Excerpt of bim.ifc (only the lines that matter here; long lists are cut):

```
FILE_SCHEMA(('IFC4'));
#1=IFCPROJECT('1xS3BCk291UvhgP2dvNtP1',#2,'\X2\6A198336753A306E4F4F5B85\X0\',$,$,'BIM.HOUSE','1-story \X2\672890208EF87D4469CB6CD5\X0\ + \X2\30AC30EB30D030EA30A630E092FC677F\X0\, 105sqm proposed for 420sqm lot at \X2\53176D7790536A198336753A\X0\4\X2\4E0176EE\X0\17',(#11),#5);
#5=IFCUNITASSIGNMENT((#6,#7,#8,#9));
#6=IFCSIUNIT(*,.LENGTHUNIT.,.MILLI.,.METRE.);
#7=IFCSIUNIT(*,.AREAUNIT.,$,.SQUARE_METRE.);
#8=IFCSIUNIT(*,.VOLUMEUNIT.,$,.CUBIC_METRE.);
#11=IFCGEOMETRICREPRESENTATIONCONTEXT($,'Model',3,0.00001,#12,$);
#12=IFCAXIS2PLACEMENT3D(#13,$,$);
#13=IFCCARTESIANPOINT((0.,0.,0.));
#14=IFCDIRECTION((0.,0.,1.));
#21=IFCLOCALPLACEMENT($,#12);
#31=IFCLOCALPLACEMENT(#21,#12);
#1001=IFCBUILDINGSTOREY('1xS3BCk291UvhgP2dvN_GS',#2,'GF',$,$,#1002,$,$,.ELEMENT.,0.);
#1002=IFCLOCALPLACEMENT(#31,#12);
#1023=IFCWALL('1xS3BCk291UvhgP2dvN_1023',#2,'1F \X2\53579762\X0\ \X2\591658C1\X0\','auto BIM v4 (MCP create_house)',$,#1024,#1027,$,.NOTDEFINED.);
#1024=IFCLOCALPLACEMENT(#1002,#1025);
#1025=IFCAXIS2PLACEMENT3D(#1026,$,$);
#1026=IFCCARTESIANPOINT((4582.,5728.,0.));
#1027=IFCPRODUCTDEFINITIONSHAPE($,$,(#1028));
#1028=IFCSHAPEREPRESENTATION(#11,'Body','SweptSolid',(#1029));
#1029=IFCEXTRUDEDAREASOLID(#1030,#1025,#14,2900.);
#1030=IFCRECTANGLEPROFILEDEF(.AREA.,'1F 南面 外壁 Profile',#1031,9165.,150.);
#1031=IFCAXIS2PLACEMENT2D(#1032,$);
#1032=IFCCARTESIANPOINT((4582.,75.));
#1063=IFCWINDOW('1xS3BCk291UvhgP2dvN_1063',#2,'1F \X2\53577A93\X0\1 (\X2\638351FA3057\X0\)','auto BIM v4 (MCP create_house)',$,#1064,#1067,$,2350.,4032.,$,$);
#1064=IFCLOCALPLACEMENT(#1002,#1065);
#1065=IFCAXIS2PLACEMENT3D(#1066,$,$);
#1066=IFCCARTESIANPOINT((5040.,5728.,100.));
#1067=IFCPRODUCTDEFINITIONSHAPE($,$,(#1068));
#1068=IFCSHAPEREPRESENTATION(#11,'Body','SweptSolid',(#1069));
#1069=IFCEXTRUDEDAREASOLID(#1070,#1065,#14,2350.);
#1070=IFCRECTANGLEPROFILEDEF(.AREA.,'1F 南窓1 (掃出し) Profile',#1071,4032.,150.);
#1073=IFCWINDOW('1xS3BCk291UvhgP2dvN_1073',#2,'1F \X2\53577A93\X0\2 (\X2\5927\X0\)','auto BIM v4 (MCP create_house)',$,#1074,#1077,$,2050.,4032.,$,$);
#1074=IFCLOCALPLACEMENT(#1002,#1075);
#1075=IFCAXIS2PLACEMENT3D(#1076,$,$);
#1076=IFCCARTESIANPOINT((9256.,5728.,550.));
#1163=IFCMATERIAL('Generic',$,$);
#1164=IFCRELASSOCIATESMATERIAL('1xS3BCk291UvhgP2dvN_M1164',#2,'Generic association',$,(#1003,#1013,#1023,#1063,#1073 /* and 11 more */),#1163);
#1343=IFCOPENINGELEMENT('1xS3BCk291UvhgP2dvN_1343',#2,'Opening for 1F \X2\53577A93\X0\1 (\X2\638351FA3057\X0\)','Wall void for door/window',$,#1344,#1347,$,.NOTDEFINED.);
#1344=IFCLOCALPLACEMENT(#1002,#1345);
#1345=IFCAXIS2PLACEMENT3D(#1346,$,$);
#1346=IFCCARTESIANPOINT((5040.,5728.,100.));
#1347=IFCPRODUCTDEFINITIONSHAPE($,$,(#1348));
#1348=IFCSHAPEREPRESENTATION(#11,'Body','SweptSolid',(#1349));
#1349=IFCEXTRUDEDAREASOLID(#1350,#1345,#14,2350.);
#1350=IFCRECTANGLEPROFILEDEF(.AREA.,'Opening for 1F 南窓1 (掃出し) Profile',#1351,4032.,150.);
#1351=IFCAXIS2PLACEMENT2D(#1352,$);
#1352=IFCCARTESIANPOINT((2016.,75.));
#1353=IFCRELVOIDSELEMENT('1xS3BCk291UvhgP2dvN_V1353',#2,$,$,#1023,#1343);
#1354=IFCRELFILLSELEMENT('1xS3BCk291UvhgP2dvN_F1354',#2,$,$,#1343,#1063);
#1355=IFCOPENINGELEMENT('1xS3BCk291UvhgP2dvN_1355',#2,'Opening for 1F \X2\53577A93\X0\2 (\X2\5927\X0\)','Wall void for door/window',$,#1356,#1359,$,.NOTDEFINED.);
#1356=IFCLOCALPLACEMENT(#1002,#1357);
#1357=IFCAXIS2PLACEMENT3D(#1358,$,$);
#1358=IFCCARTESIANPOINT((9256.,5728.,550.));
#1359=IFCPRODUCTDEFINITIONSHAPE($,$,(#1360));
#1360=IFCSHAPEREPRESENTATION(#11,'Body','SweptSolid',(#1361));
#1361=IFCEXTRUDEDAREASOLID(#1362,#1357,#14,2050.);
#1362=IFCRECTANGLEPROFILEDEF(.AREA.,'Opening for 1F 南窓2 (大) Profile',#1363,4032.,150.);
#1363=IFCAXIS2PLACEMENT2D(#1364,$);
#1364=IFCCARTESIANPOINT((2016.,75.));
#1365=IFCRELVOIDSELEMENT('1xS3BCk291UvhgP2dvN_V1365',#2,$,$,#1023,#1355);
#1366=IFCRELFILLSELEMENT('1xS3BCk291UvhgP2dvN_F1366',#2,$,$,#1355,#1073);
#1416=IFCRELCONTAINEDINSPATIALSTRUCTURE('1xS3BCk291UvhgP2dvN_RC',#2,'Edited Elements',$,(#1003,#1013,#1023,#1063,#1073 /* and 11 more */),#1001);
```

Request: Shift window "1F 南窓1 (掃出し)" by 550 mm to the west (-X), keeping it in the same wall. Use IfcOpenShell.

```python
import ifcopenshell
import ifcopenshell.api.geometry
import ifcopenshell.util.placement

model = ifcopenshell.open("bim.ifc")

window = model.by_id(1063)
opening = window.FillsVoids[0].RelatingOpeningElement
wall = opening.VoidsElements[0].RelatingBuildingElement

wall_matrix = ifcopenshell.util.placement.get_local_placement(wall.ObjectPlacement)
shift = wall_matrix[:3, 0] * -550.0
before = ifcopenshell.util.placement.get_local_placement(window.ObjectPlacement)[:3, 3].copy()

# The window is not placed relative to its opening, so move both.
for product in (opening, window):
    matrix = ifcopenshell.util.placement.get_local_placement(product.ObjectPlacement)
    matrix[:3, 3] += shift
    ifcopenshell.api.geometry.edit_object_placement(model, product=product, matrix=matrix, is_si=False)

after = ifcopenshell.util.placement.get_local_placement(window.ObjectPlacement)[:3, 3]
print("window moved by", (after - before).round(3) + 0.0)

model.write("bim_edited.ifc")
```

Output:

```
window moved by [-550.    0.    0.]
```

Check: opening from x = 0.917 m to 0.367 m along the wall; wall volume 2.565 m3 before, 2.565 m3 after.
